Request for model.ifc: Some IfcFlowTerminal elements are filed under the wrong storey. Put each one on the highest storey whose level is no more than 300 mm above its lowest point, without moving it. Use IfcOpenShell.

First a look at what the model holds.

```python
import ifcopenshell
import ifcopenshell.util.element
import ifcopenshell.util.placement

model = ifcopenshell.open("model.ifc")
print(model.schema)
for storey in model.by_type("IfcBuildingStorey"):
    level = ifcopenshell.util.placement.get_storey_elevation(storey)
    count = sum(e.is_a("IfcFlowTerminal") for e in ifcopenshell.util.element.get_contained(storey))
    print(storey.id(), storey.Name, round(level, 3), count, sep=" | ")
```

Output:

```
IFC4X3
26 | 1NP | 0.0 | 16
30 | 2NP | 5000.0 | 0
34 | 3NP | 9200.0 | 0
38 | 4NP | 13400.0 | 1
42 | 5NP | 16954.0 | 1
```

```python
import ifcopenshell
import ifcopenshell.api.spatial
import ifcopenshell.geom
import ifcopenshell.util.element
import ifcopenshell.util.placement
import ifcopenshell.util.shape
import ifcopenshell.util.unit

model = ifcopenshell.open("model.ifc")
unit_scale = ifcopenshell.util.unit.calculate_unit_scale(model)
settings = ifcopenshell.geom.settings()

levels = sorted(
    ((ifcopenshell.util.placement.get_storey_elevation(s) * unit_scale, s) for s in model.by_type("IfcBuildingStorey")),
    key=lambda pair: pair[0],
)

for e in model.by_type("IfcFlowTerminal"):
    current = e.ContainedInStructure[0].RelatingStructure if e.ContainedInStructure else None
    if current is None or not current.is_a("IfcBuildingStorey"):
        continue
    shape = ifcopenshell.geom.create_shape(settings, e)
    bottom = ifcopenshell.util.shape.get_shape_bottom_elevation(shape, shape.geometry)
    below = [s for level, s in levels if level <= bottom + 0.3]
    storey = below[-1] if below else levels[0][1]
    if storey != current:
        # assign_container keeps the world position.
        ifcopenshell.api.spatial.assign_container(model, products=[e], relating_structure=storey)
        print(e.id(), current.Name, "->", storey.Name)

model.write("model_edited.ifc")
```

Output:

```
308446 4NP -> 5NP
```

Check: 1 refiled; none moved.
